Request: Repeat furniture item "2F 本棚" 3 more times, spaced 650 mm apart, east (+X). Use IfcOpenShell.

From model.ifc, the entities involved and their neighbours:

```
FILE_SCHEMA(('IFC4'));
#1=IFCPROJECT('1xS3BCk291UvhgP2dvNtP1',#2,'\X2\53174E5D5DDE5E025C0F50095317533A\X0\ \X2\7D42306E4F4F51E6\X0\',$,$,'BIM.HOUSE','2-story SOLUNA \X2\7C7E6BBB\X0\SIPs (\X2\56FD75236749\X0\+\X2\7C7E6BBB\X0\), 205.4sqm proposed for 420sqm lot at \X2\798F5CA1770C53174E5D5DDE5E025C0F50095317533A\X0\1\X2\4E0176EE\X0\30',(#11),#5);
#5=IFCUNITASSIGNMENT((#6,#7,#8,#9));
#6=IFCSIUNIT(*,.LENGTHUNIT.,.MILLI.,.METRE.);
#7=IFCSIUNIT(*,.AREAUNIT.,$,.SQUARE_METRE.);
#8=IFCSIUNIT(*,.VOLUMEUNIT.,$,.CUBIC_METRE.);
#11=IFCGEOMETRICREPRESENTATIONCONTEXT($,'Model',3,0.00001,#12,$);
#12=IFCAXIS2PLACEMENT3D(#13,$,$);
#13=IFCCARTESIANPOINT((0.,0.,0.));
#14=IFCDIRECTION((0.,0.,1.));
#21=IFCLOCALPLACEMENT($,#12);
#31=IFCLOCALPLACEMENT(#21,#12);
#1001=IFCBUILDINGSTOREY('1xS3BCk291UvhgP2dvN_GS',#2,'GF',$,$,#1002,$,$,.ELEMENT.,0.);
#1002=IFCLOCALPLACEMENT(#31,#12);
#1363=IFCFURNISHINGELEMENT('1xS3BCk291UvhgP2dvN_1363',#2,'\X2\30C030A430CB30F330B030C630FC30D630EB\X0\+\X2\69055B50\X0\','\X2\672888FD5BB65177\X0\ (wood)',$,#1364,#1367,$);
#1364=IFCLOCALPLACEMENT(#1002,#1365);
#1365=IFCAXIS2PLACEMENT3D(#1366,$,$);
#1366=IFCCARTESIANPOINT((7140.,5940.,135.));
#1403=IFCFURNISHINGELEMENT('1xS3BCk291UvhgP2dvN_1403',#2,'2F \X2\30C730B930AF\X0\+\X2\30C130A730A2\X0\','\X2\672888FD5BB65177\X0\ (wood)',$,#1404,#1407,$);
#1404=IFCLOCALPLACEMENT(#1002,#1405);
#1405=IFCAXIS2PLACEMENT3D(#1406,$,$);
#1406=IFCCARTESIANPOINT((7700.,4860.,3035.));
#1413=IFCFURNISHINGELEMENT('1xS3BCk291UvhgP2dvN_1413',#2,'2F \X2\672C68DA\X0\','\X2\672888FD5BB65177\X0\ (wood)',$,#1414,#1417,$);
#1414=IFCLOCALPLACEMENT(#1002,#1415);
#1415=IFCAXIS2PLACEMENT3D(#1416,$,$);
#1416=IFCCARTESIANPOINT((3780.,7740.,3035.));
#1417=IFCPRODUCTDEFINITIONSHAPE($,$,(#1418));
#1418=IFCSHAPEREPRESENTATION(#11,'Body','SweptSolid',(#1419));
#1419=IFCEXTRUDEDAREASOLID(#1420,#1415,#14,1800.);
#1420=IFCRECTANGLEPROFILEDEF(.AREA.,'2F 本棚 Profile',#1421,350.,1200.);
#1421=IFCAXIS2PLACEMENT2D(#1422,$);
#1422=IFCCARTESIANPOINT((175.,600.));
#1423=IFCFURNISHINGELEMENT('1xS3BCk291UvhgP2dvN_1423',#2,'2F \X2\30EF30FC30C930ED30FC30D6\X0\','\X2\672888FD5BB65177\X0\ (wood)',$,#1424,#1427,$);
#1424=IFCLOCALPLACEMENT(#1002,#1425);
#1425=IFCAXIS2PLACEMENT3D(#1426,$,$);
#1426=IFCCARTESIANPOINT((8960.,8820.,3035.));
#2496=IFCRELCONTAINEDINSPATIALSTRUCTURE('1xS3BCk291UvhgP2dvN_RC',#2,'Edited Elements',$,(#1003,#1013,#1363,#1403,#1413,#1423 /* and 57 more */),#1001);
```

```python
import numpy as np
import ifcopenshell
import ifcopenshell.api.geometry
import ifcopenshell.api.root
import ifcopenshell.util.element
import ifcopenshell.util.placement
import ifcopenshell.util.unit

model = ifcopenshell.open("model.ifc")
unit_scale = ifcopenshell.util.unit.calculate_unit_scale(model)


def reuse_history(source, copy):
    """copy_class also copies each property set's owner history, people and application; keep the originals."""
    for rel in copy.IsDefinedBy:
        if rel.is_a("IfcRelDefinesByProperties") and (history := rel.RelatingPropertyDefinition.OwnerHistory):
            rel.RelatingPropertyDefinition.OwnerHistory = source.OwnerHistory
            ifcopenshell.util.element.remove_deep2(model, history)


source = model.by_id(1413)
base = ifcopenshell.util.placement.get_local_placement(source.ObjectPlacement)
step = np.array([1.0, 0.0, 0.0]) * 0.65 / unit_scale

for i in range(1, 4):
    copy = ifcopenshell.api.root.copy_class(model, product=source)
    copy.Representation = ifcopenshell.util.element.copy_deep(
        model, source.Representation, exclude=["IfcGeometricRepresentationContext", "IfcRepresentationMap"]
    )
    reuse_history(source, copy)
    matrix = base.copy()
    matrix[:3, 3] += i * step
    print("added at", matrix[:3, 3].round(3) + 0.0)
    ifcopenshell.api.geometry.edit_object_placement(model, product=copy, matrix=matrix, is_si=False)

model.write("model_edited.ifc")
```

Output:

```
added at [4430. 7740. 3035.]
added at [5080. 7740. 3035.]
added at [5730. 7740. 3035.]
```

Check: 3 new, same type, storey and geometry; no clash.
